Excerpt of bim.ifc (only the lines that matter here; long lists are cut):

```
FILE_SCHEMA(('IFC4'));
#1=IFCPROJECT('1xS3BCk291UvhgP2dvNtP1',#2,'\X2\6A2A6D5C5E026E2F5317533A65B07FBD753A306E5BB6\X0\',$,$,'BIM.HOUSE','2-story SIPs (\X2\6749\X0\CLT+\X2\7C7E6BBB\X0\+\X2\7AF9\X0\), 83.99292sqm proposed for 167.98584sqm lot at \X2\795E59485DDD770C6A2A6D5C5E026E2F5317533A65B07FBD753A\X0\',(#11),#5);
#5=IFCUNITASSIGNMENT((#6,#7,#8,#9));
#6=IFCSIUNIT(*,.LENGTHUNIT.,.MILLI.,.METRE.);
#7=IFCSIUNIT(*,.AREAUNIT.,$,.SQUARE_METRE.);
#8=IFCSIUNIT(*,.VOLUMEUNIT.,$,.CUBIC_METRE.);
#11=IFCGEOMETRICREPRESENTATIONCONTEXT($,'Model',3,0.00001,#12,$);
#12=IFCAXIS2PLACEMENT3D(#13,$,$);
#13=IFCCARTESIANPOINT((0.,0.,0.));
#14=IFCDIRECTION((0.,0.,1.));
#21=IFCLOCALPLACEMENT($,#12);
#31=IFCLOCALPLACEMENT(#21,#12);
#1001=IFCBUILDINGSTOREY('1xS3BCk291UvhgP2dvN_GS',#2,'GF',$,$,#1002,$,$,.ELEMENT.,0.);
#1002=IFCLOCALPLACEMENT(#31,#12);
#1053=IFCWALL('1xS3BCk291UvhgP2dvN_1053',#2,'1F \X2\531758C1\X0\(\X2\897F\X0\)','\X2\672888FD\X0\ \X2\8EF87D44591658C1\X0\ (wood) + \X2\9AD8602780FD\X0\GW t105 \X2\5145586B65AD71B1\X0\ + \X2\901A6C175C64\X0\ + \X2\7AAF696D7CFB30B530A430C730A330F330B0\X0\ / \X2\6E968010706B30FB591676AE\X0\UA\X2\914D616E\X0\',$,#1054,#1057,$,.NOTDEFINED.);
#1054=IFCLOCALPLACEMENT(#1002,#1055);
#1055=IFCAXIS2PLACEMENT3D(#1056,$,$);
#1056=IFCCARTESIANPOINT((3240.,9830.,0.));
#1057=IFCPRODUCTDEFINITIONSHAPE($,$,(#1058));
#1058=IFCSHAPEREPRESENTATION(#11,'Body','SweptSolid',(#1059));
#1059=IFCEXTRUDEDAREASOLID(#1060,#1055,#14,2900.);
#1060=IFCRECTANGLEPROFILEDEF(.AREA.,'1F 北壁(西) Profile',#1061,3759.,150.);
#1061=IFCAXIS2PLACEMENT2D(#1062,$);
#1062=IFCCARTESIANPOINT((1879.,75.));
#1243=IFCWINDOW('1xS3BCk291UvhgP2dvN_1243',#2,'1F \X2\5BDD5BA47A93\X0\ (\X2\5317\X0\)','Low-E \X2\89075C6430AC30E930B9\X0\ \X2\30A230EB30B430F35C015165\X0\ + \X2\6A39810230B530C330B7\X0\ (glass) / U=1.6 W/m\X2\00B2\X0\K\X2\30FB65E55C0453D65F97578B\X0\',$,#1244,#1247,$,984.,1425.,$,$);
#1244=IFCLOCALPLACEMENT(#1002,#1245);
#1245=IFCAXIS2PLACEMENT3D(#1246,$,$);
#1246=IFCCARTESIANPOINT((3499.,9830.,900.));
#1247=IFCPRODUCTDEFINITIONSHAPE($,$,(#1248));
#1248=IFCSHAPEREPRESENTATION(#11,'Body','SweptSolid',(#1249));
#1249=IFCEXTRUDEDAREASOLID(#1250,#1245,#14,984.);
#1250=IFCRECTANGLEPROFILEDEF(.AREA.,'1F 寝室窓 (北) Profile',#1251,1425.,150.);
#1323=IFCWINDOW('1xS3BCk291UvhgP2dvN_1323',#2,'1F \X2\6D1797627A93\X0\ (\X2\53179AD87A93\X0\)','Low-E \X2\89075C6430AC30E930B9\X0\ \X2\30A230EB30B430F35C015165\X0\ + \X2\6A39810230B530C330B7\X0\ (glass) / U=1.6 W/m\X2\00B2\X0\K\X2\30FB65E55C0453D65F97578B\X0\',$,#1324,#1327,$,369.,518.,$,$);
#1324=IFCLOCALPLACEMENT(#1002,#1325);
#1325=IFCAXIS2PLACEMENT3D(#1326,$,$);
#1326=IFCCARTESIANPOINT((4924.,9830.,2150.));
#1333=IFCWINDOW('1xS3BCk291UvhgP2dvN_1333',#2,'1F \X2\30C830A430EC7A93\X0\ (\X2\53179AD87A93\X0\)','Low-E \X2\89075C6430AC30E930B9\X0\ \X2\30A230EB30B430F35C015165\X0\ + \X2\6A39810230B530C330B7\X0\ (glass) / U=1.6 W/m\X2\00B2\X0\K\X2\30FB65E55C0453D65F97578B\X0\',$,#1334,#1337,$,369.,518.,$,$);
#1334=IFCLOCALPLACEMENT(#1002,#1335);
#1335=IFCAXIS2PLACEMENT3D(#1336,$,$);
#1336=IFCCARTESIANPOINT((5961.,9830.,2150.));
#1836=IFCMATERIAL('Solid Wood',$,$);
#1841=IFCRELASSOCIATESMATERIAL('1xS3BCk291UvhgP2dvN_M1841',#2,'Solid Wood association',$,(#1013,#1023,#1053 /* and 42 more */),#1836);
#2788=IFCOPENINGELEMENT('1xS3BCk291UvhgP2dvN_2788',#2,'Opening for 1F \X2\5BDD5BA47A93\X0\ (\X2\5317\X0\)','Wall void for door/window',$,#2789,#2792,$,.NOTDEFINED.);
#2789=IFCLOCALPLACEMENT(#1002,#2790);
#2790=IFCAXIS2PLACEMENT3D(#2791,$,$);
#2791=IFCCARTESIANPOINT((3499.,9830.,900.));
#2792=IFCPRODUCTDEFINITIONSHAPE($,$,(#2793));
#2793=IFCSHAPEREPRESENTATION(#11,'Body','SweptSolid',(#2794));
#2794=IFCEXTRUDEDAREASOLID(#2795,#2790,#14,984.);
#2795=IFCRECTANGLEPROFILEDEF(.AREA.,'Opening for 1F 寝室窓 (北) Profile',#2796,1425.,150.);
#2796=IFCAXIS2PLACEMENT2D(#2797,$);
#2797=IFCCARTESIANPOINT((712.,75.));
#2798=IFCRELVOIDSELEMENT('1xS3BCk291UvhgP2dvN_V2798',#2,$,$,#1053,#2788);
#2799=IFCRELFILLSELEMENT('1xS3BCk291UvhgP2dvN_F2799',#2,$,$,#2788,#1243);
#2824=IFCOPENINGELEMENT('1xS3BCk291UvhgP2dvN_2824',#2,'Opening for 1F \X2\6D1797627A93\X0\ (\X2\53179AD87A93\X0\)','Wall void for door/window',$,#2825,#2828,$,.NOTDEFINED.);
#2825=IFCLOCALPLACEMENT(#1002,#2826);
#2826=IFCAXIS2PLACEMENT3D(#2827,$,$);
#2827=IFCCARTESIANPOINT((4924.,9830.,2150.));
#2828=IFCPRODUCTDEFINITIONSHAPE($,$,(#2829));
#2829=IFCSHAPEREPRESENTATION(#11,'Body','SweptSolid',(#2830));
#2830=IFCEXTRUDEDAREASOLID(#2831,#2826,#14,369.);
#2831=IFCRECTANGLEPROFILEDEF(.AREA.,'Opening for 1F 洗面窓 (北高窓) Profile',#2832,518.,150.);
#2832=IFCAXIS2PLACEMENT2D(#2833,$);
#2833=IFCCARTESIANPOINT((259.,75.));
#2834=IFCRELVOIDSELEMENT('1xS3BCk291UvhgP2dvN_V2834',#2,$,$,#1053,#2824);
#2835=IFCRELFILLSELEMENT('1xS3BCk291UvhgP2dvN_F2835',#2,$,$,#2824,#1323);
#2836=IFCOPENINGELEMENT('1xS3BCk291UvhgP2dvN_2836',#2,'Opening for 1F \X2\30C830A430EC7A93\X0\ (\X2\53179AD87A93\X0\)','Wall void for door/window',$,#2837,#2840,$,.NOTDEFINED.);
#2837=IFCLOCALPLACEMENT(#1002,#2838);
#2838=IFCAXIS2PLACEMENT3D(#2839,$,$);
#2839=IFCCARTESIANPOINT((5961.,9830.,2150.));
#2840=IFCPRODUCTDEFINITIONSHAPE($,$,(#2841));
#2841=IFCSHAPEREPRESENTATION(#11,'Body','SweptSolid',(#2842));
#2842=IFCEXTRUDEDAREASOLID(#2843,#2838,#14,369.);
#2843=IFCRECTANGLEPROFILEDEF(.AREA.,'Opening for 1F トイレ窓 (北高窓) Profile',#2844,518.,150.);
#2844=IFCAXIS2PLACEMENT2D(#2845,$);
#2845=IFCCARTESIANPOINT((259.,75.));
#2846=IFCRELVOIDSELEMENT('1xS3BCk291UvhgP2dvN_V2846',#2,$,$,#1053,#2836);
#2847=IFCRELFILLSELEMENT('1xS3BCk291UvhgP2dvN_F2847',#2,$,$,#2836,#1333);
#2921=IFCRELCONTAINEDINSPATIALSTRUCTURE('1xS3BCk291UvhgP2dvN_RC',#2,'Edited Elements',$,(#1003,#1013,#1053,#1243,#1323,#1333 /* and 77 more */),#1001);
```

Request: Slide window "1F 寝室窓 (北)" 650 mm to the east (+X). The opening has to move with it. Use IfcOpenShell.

```python
import ifcopenshell
import ifcopenshell.api.geometry
import ifcopenshell.util.placement

model = ifcopenshell.open("bim.ifc")

window = model.by_guid("1xS3BCk291UvhgP2dvN_1243")
opening = window.FillsVoids[0].RelatingOpeningElement
wall = opening.VoidsElements[0].RelatingBuildingElement

wall_matrix = ifcopenshell.util.placement.get_local_placement(wall.ObjectPlacement)
shift = wall_matrix[:3, 0] * 650.0
before = ifcopenshell.util.placement.get_local_placement(window.ObjectPlacement)[:3, 3].copy()

# The window is not placed relative to its opening, so move both.
for product in (opening, window):
    matrix = ifcopenshell.util.placement.get_local_placement(product.ObjectPlacement)
    matrix[:3, 3] += shift
    ifcopenshell.api.geometry.edit_object_placement(model, product=product, matrix=matrix, is_si=False)

after = ifcopenshell.util.placement.get_local_placement(window.ObjectPlacement)[:3, 3]
print("window moved by", (after - before).round(3) + 0.0)

model.write("bim_edited.ifc")
```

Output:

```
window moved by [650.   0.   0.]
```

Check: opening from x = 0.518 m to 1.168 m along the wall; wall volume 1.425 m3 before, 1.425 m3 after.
